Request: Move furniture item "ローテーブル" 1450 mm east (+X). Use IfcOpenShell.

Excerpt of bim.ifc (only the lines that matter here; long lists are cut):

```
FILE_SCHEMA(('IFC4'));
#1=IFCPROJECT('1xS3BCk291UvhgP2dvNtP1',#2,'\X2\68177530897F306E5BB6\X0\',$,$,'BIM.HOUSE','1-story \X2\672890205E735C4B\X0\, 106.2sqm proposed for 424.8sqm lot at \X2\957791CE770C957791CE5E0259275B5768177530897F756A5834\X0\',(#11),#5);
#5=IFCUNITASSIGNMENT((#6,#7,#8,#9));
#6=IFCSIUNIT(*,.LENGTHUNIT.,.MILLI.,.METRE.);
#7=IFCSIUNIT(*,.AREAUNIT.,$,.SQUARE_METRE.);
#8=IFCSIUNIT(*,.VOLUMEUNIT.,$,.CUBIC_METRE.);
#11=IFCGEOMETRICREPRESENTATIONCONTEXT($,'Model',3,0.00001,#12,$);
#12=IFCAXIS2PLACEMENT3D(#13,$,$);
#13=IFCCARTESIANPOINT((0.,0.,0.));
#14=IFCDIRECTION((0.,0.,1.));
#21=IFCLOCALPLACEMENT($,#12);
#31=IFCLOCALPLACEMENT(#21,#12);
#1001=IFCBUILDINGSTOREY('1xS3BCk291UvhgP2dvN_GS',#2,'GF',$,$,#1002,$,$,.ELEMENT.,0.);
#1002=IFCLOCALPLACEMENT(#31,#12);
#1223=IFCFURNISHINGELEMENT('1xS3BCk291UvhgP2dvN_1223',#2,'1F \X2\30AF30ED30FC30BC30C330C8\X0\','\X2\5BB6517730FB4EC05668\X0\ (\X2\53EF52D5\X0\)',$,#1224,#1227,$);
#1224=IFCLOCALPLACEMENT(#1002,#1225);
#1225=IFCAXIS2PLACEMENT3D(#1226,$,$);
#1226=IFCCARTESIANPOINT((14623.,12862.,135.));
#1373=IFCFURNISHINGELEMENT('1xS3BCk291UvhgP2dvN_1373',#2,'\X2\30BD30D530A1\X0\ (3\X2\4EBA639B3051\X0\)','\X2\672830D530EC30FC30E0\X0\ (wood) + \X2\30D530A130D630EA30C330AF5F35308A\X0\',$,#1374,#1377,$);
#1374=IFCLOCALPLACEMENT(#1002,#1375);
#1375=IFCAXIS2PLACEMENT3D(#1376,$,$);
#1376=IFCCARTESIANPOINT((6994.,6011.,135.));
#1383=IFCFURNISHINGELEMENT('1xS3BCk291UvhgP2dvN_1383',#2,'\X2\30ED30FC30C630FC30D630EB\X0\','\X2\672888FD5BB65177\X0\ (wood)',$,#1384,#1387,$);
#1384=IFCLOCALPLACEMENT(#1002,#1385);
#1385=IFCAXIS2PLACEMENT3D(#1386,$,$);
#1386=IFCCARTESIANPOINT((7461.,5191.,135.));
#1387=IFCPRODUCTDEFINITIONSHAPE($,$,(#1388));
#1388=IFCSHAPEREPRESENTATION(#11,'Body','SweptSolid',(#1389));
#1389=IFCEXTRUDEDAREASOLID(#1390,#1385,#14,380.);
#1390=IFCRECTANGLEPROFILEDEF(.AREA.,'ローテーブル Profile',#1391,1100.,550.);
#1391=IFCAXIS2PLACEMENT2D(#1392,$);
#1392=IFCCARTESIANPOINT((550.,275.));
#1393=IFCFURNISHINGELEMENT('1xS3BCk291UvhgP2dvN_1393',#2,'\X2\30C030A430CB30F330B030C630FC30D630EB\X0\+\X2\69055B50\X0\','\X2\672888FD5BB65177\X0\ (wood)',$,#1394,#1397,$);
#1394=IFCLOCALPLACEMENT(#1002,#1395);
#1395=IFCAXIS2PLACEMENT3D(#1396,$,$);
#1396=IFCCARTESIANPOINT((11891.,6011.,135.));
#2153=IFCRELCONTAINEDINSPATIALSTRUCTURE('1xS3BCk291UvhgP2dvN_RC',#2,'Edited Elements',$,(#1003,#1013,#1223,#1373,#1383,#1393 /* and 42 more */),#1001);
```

```python
import ifcopenshell
import ifcopenshell.api.geometry
import ifcopenshell.util.placement
import ifcopenshell.util.unit

model = ifcopenshell.open("bim.ifc")
unit_scale = ifcopenshell.util.unit.calculate_unit_scale(model)

item = model.by_guid("1xS3BCk291UvhgP2dvN_1383")
matrix = ifcopenshell.util.placement.get_local_placement(item.ObjectPlacement)
matrix[0, 3] += 1.45 / unit_scale
ifcopenshell.api.geometry.edit_object_placement(model, product=item, matrix=matrix, is_si=False)

print(ifcopenshell.util.placement.get_local_placement(item.ObjectPlacement).round(3) + 0.0)

model.write("bim_updated.ifc")
```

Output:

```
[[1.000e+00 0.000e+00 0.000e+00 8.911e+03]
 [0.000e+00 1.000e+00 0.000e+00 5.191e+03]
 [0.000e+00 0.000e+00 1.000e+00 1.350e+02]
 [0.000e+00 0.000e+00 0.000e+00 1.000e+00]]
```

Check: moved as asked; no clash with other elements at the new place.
